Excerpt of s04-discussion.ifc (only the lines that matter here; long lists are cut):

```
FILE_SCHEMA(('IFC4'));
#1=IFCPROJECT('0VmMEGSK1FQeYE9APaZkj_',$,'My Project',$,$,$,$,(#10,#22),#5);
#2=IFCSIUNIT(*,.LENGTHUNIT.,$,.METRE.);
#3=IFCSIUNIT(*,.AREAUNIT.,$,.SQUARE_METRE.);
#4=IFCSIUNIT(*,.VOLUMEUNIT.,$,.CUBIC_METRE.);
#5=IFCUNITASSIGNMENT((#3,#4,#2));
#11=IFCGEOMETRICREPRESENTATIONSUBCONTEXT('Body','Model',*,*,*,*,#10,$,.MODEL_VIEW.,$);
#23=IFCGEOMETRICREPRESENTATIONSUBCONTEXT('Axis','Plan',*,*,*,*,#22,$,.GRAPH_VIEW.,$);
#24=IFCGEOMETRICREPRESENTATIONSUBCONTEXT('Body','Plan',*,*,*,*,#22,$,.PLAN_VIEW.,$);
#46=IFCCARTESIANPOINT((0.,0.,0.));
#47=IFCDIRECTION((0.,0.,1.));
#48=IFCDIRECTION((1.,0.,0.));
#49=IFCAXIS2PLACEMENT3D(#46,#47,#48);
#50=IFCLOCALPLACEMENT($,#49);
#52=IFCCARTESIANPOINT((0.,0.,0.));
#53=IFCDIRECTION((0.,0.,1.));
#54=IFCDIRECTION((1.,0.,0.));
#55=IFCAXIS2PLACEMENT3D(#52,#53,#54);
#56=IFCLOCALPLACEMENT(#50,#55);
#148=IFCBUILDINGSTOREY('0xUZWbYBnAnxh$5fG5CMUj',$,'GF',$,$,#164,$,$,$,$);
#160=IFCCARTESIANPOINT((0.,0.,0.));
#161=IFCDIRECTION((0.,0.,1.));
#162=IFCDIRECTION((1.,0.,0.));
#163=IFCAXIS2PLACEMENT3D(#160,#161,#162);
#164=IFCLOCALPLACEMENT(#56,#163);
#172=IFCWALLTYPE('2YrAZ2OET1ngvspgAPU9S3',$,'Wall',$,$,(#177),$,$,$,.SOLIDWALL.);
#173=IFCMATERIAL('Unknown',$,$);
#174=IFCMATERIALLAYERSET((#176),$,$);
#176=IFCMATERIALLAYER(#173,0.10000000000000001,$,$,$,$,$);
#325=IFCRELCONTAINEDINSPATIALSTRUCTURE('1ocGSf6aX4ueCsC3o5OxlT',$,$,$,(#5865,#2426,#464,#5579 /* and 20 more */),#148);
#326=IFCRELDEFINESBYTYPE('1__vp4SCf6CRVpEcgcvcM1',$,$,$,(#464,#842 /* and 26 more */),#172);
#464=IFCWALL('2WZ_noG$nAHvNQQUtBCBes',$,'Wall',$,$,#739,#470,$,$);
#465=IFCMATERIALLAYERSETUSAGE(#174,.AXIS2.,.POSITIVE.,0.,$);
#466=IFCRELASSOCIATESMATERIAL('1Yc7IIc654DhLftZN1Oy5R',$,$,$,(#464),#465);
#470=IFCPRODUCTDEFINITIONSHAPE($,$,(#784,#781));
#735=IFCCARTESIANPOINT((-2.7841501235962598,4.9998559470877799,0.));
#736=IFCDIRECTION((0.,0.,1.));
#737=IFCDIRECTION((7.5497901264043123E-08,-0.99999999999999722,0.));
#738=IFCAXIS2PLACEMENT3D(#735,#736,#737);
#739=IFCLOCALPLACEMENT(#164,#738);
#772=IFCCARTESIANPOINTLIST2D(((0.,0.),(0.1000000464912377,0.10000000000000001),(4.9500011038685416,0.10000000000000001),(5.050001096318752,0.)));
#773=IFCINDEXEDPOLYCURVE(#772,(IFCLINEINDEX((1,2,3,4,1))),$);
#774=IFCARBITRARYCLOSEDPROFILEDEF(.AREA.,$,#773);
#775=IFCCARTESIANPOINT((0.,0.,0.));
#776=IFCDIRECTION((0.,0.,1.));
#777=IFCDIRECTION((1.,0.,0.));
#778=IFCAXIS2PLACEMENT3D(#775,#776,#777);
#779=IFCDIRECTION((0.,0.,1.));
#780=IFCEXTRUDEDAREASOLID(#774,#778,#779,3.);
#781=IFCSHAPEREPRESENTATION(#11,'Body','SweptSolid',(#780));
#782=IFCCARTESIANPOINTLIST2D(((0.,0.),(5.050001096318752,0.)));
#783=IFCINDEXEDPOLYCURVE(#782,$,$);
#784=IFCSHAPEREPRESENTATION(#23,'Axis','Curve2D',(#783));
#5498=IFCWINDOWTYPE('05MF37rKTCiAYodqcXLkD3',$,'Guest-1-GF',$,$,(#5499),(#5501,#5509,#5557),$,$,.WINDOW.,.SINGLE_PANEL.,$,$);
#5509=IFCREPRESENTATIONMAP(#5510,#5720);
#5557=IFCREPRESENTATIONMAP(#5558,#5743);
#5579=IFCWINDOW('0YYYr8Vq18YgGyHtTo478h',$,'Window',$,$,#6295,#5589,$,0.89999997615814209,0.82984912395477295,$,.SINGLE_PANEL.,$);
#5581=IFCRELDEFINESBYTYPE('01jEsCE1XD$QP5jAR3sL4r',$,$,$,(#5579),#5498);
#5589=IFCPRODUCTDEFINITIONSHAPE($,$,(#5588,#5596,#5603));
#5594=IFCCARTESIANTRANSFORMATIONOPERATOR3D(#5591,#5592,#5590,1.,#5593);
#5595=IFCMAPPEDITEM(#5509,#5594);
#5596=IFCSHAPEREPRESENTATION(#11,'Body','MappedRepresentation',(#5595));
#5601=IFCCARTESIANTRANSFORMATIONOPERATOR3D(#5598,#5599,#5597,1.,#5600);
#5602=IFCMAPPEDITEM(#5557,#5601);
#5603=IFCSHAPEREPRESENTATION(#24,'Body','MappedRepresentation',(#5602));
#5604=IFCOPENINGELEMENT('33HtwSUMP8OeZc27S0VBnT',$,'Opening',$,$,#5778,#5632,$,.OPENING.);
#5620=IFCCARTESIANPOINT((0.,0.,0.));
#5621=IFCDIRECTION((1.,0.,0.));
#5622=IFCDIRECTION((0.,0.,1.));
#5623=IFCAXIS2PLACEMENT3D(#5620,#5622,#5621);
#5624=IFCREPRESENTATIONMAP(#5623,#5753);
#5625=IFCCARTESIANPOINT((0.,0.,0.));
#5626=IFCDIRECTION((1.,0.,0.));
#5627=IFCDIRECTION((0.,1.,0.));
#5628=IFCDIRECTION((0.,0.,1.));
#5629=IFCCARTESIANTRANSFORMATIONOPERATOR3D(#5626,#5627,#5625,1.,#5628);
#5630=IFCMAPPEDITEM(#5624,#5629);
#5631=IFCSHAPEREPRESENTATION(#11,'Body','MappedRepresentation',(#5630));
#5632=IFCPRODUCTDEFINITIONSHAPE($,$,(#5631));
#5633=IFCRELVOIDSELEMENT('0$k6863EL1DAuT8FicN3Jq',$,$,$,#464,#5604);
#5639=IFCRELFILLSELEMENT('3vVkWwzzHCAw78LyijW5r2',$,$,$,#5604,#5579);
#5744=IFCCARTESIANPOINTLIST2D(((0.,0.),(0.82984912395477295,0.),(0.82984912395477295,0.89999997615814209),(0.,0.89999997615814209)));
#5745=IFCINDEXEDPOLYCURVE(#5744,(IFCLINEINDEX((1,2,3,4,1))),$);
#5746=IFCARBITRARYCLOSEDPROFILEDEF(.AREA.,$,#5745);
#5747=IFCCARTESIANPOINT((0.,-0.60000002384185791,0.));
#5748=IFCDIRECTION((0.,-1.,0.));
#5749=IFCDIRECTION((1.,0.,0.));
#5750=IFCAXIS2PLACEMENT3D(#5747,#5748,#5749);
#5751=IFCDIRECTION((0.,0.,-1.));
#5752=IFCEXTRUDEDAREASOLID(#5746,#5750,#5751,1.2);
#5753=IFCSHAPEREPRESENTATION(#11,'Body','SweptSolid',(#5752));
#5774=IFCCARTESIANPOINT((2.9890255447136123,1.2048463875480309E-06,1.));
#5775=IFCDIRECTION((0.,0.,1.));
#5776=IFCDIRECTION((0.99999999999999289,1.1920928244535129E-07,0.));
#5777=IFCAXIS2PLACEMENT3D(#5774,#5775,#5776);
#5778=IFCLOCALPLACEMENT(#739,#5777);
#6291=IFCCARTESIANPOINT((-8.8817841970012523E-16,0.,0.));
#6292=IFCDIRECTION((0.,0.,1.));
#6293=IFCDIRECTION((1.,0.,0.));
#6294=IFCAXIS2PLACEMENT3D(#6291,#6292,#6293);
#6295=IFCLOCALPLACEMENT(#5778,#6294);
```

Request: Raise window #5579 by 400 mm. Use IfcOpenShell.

```python
import numpy as np
import ifcopenshell
import ifcopenshell.api.geometry
import ifcopenshell.util.placement
import ifcopenshell.util.unit

model = ifcopenshell.open("s04-discussion.ifc")
unit_scale = ifcopenshell.util.unit.calculate_unit_scale(model)

window = model.by_guid("0YYYr8Vq18YgGyHtTo478h")
opening = window.FillsVoids[0].RelatingOpeningElement
dz = 0.4 / unit_scale

shift = np.array([0.0, 0.0, dz])
# The window is placed relative to its opening, so it follows when the opening moves.
matrix = ifcopenshell.util.placement.get_local_placement(opening.ObjectPlacement)
matrix[:3, 3] += shift
ifcopenshell.api.geometry.edit_object_placement(
    model, product=opening, matrix=matrix, is_si=False, should_transform_children=True
)

print(f"moved by {dz * unit_scale:+.3f} m")

model.write("s04-discussion-out.ifc")
```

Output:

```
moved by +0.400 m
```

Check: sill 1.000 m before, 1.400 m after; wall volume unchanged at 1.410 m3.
